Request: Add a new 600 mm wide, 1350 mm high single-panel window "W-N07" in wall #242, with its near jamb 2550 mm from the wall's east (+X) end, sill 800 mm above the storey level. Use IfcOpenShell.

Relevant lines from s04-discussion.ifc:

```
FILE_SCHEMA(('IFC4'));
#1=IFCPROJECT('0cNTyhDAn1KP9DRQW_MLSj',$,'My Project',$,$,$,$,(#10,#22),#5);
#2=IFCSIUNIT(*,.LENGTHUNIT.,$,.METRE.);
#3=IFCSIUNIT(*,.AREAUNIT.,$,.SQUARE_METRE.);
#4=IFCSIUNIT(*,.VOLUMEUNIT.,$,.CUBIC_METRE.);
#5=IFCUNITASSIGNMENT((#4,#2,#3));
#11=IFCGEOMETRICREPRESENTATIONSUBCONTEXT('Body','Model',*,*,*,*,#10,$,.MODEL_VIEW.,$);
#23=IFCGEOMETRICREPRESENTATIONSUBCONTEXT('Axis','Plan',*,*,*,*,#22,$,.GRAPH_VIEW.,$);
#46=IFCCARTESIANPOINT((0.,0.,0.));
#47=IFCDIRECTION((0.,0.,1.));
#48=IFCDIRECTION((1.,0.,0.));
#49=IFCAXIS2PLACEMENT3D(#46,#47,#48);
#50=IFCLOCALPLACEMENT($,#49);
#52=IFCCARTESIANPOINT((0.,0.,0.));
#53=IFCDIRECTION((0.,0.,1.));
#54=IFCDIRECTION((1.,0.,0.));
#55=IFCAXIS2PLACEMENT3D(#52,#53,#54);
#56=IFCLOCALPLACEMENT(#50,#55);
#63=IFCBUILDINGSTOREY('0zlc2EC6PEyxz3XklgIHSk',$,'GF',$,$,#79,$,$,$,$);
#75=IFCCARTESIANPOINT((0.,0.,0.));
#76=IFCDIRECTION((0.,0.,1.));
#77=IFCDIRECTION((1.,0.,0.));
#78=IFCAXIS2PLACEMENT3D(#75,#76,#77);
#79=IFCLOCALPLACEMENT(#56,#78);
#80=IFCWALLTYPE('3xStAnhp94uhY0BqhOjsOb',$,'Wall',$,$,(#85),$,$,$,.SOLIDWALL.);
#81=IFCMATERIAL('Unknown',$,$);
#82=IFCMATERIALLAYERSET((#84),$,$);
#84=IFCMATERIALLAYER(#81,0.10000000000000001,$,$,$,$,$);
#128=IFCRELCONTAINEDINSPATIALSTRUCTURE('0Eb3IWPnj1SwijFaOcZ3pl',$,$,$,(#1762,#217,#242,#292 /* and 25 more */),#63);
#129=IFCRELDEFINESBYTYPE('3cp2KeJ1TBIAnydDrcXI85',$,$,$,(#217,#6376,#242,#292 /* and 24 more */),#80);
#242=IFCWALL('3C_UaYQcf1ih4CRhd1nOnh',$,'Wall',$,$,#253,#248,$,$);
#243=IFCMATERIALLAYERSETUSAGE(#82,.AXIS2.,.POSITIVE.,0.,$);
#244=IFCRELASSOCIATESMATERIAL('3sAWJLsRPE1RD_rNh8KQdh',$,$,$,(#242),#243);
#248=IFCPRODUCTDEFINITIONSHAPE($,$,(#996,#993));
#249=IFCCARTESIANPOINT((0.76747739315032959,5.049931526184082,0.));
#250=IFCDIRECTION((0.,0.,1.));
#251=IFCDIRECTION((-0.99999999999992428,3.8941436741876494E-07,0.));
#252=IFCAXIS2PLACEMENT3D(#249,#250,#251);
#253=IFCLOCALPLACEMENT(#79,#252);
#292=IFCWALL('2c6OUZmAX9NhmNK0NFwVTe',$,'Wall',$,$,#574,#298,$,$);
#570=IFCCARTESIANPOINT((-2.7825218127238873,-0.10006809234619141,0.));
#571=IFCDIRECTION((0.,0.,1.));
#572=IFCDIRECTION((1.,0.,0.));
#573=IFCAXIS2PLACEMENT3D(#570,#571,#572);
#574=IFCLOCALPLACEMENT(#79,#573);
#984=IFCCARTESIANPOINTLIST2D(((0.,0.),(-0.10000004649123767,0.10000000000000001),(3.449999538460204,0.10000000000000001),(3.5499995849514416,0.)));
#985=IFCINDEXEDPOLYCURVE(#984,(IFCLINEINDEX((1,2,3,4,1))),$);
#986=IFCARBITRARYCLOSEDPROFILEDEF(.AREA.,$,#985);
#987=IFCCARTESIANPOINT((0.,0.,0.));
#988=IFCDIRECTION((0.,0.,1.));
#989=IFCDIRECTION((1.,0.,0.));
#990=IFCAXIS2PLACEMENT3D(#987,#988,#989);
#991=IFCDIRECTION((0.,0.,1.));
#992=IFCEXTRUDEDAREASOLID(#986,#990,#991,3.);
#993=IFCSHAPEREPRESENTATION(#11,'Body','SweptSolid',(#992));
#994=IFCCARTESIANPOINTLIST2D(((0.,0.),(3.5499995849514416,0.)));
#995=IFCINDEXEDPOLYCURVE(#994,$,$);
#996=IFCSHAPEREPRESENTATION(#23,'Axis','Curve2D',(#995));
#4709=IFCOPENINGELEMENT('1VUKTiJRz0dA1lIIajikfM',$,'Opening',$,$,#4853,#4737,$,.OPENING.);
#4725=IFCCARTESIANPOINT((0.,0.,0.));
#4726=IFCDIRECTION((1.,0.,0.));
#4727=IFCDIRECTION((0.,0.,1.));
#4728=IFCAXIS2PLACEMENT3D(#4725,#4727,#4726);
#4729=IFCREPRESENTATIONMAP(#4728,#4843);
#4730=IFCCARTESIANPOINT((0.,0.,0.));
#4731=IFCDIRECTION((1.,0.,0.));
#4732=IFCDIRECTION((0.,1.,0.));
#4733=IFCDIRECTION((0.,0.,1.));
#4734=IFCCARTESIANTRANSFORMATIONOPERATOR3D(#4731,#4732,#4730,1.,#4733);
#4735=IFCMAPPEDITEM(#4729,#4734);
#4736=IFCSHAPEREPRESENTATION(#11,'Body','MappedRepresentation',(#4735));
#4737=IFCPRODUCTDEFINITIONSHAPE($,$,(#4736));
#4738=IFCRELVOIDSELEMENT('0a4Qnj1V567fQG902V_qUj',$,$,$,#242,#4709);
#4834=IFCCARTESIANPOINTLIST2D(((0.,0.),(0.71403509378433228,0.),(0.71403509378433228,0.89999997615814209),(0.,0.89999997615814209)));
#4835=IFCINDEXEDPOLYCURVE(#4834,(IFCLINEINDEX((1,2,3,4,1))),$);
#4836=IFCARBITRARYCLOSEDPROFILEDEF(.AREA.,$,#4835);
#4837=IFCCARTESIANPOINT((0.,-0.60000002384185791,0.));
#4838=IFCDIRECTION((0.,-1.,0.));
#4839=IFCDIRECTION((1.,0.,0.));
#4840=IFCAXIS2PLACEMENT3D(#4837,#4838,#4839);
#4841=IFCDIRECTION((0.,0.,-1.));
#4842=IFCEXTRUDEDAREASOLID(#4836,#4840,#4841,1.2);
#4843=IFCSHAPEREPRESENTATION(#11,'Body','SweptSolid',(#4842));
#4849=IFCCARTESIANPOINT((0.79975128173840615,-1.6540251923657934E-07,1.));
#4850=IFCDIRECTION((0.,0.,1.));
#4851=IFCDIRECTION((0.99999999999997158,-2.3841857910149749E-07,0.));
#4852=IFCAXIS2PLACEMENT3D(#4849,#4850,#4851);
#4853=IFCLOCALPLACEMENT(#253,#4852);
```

```python
import numpy as np
import ifcopenshell
import ifcopenshell.api.feature
import ifcopenshell.api.geometry
import ifcopenshell.api.root
import ifcopenshell.api.spatial
import ifcopenshell.geom
import ifcopenshell.util.element
import ifcopenshell.util.placement
import ifcopenshell.util.representation
import ifcopenshell.util.shape
import ifcopenshell.util.unit

model = ifcopenshell.open("s04-discussion.ifc")
unit_scale = ifcopenshell.util.unit.calculate_unit_scale(model)
settings = ifcopenshell.geom.settings()


def volume(element):
    """Net volume in cubic metres, openings subtracted."""
    shape = ifcopenshell.geom.create_shape(settings, element)
    return ifcopenshell.util.shape.get_volume(shape.geometry)


wall = model.by_guid("3C_UaYQcf1ih4CRhd1nOnh")
storey = ifcopenshell.util.element.get_container(wall, ifc_class="IfcBuildingStorey")
context = ifcopenshell.util.representation.get_context(model, "Model", "Body", "MODEL_VIEW")
before = volume(wall)

width, height, from_end, sill = 0.6, 1.35, 2.55, 0.8  # metres

# The wall runs along its own X axis, and the end named is its -X end.
wall_shape = ifcopenshell.geom.create_shape(settings, wall)
x, y, z = ifcopenshell.util.shape.get_vertices(wall_shape.geometry).T
start = x.min() + from_end
face, thickness = float(y.min()), float(y.max() - y.min())
wall_matrix = ifcopenshell.util.placement.get_local_placement(wall.ObjectPlacement)
level = ifcopenshell.util.placement.get_local_placement(storey.ObjectPlacement)[2, 3]


def in_wall(x, y):
    """Placement at x, y metres in the wall's axes, at sill height."""
    matrix = wall_matrix.copy()
    matrix[:, 3] = wall_matrix @ np.array([x / unit_scale, y / unit_scale, 0.0, 1.0])
    matrix[2, 3] = level + sill / unit_scale
    return matrix


# Opening: a box that overshoots both wall faces by 50 mm.
opening = ifcopenshell.api.root.create_entity(model, ifc_class="IfcOpeningElement", predefined_type="OPENING")
box = ifcopenshell.api.geometry.add_wall_representation(
    model, context=context, length=width, height=height, thickness=thickness + 0.1
)
ifcopenshell.api.geometry.assign_representation(model, product=opening, representation=box)
ifcopenshell.api.geometry.edit_object_placement(model, product=opening, matrix=in_wall(start, face - 0.05), is_si=False)
ifcopenshell.api.feature.add_feature(model, feature=opening, element=wall)

window = ifcopenshell.api.root.create_entity(model, ifc_class="IfcWindow", name="W-N07", predefined_type="WINDOW")
window.OverallWidth, window.OverallHeight = width / unit_scale, height / unit_scale
window.PartitioningType = "SINGLE_PANEL"
body = ifcopenshell.api.geometry.add_window_representation(
    model,
    context=context,
    overall_width=window.OverallWidth,
    overall_height=window.OverallHeight,
    partition_type="SINGLE_PANEL",
)
ifcopenshell.api.geometry.assign_representation(model, product=window, representation=body)
ifcopenshell.api.spatial.assign_container(model, products=[window], relating_structure=storey)
ifcopenshell.api.feature.add_filling(model, opening=opening, element=window)

# Centre the window in the wall's thickness.
ifcopenshell.api.geometry.edit_object_placement(model, product=window, matrix=in_wall(start, face), is_si=False)
window_shape = ifcopenshell.geom.create_shape(settings, window)
depth = ifcopenshell.util.shape.get_vertices(window_shape.geometry)[:, 1]
offset = face + thickness / 2 - (depth.min() + depth.max()) / 2
ifcopenshell.api.geometry.edit_object_placement(model, product=window, matrix=in_wall(start, offset), is_si=False)

after = volume(wall)

print(f"wall volume {before:.3f} -> {after:.3f} m3")

model.write("s04-discussion_edited.ifc")
```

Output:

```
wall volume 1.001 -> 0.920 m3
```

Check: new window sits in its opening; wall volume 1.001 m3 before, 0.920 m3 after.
